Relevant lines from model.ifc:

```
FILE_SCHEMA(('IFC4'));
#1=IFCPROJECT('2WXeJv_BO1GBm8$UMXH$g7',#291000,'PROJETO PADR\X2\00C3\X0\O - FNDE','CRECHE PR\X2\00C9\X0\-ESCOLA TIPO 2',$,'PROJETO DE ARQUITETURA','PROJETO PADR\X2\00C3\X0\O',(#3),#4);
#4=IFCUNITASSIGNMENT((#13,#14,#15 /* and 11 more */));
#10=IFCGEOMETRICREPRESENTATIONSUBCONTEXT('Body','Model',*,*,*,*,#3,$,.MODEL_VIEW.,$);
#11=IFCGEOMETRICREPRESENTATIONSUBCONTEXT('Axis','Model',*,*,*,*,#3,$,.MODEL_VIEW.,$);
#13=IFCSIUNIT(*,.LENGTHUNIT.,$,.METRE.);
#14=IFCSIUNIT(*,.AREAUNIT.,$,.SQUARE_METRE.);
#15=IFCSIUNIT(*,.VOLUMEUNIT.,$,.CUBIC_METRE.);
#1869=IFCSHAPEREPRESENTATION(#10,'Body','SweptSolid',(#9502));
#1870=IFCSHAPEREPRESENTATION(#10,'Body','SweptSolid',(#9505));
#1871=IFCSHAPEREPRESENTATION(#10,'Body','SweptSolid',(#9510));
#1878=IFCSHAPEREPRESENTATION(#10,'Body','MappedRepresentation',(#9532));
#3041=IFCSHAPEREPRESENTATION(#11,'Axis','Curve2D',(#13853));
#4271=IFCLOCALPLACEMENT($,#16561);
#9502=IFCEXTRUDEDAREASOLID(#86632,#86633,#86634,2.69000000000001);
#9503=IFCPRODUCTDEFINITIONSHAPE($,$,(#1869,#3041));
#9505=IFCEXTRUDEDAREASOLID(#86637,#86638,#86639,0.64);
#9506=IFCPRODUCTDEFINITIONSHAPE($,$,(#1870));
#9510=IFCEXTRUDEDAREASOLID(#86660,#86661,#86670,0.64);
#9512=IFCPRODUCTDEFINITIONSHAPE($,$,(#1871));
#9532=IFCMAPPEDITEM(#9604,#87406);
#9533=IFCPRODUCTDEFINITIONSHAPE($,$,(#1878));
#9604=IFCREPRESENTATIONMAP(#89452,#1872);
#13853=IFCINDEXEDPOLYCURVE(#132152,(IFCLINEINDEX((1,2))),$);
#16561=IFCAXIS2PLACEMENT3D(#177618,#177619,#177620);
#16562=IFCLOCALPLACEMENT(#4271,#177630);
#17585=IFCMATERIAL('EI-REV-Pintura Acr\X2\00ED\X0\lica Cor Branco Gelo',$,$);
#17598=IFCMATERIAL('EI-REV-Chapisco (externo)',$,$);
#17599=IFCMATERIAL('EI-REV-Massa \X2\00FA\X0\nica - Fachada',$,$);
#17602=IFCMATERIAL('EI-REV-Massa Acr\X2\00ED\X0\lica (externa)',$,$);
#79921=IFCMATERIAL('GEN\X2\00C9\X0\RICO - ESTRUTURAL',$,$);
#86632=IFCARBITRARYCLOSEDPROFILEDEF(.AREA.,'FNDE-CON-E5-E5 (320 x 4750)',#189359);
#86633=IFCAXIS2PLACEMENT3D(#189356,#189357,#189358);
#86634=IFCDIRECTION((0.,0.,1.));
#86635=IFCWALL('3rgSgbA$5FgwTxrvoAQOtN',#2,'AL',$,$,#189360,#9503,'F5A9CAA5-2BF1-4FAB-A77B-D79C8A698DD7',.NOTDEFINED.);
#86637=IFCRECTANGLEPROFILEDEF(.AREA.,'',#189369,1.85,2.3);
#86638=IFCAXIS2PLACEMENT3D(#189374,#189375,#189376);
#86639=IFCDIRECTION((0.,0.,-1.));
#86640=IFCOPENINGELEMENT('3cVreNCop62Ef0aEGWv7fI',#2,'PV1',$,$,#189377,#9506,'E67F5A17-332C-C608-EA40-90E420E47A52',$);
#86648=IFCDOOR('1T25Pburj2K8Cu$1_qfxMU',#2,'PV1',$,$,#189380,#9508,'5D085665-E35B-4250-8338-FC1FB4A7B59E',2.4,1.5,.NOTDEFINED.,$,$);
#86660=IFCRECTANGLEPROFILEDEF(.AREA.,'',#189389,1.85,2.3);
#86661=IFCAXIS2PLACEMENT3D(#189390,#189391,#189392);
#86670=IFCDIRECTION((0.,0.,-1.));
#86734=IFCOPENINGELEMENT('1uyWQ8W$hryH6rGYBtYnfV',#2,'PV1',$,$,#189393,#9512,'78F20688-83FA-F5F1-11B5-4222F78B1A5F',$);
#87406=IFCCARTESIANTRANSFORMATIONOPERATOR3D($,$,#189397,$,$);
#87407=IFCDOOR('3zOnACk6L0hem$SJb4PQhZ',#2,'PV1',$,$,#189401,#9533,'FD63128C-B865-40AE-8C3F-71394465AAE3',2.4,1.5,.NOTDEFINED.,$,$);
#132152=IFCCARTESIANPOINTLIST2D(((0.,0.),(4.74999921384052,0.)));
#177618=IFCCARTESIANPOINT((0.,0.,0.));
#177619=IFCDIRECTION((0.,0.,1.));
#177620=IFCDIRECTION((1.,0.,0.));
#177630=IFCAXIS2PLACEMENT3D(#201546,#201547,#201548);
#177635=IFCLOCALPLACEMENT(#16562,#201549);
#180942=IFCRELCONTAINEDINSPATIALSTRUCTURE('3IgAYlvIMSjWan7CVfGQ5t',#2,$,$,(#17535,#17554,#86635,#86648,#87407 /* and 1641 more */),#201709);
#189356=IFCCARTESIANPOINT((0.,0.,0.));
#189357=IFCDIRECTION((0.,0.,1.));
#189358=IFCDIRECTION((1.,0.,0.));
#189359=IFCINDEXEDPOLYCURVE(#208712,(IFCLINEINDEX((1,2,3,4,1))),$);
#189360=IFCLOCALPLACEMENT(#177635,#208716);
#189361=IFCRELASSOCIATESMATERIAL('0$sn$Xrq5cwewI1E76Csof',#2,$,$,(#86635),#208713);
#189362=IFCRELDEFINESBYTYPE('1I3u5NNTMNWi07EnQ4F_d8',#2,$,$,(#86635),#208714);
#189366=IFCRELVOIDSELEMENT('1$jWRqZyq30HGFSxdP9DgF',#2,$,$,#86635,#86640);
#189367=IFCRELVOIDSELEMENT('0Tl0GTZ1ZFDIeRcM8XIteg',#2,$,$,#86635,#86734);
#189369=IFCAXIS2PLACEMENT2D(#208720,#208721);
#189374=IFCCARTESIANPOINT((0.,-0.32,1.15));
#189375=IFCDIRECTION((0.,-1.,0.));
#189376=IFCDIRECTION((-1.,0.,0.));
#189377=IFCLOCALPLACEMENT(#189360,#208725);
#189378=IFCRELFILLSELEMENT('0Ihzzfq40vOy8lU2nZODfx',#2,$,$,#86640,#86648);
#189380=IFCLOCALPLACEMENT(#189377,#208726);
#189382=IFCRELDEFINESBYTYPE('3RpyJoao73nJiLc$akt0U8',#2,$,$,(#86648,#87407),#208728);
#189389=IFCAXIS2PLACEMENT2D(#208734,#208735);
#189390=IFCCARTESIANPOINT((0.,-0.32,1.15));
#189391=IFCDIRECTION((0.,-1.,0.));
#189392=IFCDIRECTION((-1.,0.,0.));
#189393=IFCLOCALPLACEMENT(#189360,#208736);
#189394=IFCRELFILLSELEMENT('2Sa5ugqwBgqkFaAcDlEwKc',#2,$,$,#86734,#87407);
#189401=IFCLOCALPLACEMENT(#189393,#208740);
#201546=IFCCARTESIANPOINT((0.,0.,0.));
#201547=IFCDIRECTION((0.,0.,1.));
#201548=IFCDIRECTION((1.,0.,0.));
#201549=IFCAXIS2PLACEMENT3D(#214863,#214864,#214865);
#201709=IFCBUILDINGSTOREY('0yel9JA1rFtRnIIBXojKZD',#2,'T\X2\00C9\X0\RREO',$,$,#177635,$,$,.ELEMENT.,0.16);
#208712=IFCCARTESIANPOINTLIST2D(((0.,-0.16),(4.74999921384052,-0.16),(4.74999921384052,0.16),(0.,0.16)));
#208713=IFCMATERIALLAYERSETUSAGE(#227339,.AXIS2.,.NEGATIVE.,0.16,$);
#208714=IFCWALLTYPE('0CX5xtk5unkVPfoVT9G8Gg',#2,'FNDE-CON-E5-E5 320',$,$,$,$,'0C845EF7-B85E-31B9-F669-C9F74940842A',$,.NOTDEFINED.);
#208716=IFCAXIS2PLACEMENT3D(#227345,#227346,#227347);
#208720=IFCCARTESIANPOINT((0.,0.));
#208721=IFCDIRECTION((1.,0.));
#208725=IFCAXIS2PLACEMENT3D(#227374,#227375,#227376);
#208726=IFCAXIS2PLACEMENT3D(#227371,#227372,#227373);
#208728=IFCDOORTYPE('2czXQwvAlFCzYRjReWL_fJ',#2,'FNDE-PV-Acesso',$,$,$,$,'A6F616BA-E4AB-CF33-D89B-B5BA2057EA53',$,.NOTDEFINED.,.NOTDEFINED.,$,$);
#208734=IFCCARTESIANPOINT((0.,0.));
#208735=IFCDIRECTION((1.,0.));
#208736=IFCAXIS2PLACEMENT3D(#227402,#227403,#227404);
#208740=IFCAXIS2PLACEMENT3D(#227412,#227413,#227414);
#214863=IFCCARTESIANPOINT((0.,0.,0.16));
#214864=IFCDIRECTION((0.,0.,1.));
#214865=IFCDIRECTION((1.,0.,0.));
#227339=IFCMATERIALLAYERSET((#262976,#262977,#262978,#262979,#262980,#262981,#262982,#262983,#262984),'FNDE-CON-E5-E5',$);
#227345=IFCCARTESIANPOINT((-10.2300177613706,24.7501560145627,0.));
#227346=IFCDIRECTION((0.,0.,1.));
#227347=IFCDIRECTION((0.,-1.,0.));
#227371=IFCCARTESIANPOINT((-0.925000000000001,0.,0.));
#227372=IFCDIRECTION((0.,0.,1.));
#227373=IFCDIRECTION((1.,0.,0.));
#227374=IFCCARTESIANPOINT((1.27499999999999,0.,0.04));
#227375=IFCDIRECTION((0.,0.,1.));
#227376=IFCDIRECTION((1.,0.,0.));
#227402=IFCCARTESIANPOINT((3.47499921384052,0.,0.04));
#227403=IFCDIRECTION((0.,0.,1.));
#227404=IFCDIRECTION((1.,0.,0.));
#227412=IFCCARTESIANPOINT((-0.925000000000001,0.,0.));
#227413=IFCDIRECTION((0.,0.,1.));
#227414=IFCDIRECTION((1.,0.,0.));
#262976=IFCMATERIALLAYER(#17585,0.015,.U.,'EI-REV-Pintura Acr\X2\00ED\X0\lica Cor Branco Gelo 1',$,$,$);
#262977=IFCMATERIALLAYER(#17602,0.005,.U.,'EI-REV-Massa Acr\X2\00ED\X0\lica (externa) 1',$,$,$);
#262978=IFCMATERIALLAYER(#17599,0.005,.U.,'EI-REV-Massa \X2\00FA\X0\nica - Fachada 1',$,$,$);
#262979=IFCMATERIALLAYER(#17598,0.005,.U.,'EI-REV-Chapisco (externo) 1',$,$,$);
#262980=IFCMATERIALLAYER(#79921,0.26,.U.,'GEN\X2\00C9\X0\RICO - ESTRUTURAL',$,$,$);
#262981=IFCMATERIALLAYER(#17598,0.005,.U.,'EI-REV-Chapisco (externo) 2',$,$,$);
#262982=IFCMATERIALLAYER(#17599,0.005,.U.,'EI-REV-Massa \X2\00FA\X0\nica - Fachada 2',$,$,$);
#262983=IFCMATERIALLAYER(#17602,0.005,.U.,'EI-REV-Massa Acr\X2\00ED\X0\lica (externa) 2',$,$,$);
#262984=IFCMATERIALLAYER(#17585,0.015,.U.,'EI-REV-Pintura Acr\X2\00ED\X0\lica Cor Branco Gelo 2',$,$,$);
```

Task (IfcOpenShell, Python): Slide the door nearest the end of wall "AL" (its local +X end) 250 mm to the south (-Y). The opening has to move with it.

```python
import ifcopenshell
import ifcopenshell.api.geometry
import ifcopenshell.util.placement
import ifcopenshell.util.unit

model = ifcopenshell.open("model.ifc")
unit_scale = ifcopenshell.util.unit.calculate_unit_scale(model)

door = model.by_guid("3zOnACk6L0hem$SJb4PQhZ")
opening = door.FillsVoids[0].RelatingOpeningElement
wall = opening.VoidsElements[0].RelatingBuildingElement

wall_matrix = ifcopenshell.util.placement.get_local_placement(wall.ObjectPlacement)
shift = wall_matrix[:3, 0] * 0.25 / unit_scale
before = ifcopenshell.util.placement.get_local_placement(door.ObjectPlacement)[:3, 3].copy()

# The door is placed relative to its opening, so it follows when the opening moves.
matrix = ifcopenshell.util.placement.get_local_placement(opening.ObjectPlacement)
matrix[:3, 3] += shift
ifcopenshell.api.geometry.edit_object_placement(
    model, product=opening, matrix=matrix, is_si=False, should_transform_children=True
)

after = ifcopenshell.util.placement.get_local_placement(door.ObjectPlacement)[:3, 3]
print("door moved by", (after - before).round(3) + 0.0)

model.write("model_rev.ifc")
```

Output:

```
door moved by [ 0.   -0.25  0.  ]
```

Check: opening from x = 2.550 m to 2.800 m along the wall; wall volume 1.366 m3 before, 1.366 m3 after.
